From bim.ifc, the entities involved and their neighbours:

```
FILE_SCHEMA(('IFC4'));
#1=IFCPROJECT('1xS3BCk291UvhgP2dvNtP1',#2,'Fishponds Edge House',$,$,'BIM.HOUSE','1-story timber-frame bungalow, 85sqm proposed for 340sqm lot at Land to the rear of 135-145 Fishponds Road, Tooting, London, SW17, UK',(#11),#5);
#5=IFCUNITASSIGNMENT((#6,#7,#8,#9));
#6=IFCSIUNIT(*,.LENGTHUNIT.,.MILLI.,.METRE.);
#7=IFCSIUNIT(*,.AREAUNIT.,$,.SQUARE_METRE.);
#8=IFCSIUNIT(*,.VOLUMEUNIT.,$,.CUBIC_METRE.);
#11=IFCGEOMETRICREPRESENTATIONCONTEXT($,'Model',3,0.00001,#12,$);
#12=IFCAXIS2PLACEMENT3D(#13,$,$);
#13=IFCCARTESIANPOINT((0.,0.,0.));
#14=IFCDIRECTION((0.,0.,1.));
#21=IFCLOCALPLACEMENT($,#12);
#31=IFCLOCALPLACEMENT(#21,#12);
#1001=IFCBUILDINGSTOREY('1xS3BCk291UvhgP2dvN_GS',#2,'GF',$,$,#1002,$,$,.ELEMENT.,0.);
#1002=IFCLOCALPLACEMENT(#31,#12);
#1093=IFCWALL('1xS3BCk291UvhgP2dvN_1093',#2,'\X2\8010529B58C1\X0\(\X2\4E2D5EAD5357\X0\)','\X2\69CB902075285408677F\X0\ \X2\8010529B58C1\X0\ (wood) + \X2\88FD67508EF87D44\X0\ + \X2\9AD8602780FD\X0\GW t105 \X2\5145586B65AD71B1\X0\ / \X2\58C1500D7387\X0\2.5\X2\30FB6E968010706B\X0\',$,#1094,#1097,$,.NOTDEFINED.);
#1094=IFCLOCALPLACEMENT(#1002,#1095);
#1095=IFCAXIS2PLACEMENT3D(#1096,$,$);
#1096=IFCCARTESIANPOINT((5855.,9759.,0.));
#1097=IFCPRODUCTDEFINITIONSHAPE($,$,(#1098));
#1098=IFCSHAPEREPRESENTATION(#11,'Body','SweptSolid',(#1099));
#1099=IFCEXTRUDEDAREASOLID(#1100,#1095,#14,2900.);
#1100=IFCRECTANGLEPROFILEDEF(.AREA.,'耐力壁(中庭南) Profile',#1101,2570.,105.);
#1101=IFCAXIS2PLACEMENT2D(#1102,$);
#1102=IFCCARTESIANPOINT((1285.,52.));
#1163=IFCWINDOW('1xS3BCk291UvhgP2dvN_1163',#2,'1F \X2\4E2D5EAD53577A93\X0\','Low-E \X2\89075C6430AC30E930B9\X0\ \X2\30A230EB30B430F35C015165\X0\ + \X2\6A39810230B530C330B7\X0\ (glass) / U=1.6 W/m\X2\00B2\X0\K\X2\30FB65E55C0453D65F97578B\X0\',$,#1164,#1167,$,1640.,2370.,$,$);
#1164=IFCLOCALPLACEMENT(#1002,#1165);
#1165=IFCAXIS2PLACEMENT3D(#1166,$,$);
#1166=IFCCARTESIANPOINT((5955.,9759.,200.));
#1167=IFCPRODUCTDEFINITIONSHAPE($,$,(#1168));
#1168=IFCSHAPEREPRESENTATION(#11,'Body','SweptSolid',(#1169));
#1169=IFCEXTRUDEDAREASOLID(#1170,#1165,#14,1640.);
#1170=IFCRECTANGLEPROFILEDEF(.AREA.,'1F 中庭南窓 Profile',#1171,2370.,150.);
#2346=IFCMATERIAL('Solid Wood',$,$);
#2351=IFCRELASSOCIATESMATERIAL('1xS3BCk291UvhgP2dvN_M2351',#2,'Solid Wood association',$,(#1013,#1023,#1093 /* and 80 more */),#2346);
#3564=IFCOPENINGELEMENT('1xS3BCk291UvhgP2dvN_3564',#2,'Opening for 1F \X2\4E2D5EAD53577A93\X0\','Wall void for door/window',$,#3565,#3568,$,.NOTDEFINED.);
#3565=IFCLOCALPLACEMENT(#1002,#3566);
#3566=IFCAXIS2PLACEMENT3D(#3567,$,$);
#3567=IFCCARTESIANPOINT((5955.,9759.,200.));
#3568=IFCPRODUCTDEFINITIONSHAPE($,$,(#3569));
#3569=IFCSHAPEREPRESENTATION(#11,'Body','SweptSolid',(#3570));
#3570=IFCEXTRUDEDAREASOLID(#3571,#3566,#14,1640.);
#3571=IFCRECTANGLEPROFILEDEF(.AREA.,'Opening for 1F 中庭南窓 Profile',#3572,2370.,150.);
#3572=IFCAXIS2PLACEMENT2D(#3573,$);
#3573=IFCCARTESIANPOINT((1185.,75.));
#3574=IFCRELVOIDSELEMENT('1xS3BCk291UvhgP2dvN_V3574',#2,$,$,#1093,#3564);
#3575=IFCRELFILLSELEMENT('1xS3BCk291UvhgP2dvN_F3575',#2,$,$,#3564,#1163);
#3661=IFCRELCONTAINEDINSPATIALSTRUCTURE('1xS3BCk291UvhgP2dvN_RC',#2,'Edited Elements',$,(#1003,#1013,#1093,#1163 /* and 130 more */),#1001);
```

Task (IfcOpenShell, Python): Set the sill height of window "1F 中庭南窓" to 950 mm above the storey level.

```python
import numpy as np
import ifcopenshell
import ifcopenshell.api.geometry
import ifcopenshell.geom
import ifcopenshell.util.element
import ifcopenshell.util.placement
import ifcopenshell.util.shape
import ifcopenshell.util.unit

model = ifcopenshell.open("bim.ifc")
unit_scale = ifcopenshell.util.unit.calculate_unit_scale(model)

window = model.by_guid("1xS3BCk291UvhgP2dvN_1163")
opening = window.FillsVoids[0].RelatingOpeningElement
storey = ifcopenshell.util.element.get_container(window, ifc_class="IfcBuildingStorey")
level = ifcopenshell.util.placement.get_local_placement(storey.ObjectPlacement)[2, 3]

# The opening's origin need not be at the sill, so measure its lowest point.
shape = ifcopenshell.geom.create_shape(ifcopenshell.geom.settings(), opening)
bottom = ifcopenshell.util.shape.get_shape_bottom_elevation(shape, shape.geometry) / unit_scale
dz = level + 950.0 - bottom

shift = np.array([0.0, 0.0, dz])
# The window is not placed relative to its opening, so move both.
for product in (opening, window):
    matrix = ifcopenshell.util.placement.get_local_placement(product.ObjectPlacement)
    matrix[:3, 3] += shift
    ifcopenshell.api.geometry.edit_object_placement(model, product=product, matrix=matrix, is_si=False)

print(f"moved by {dz * unit_scale:+.3f} m")

model.write("bim_edited.ifc")
```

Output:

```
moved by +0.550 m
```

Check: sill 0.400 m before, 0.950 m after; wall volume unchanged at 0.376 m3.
